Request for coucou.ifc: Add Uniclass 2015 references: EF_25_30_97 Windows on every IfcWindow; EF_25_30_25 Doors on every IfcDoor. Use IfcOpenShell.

First a look at what the model holds.

```python
import ifcopenshell

model = ifcopenshell.open("coucou.ifc")
print(model.schema)
print("classifications:", [c.Name for c in model.by_type("IfcClassification")])
for ifc_class in ("IfcDoor", "IfcRoof", "IfcStair", "IfcWall", "IfcWindow"):
    print(ifc_class, len(model.by_type(ifc_class)))
```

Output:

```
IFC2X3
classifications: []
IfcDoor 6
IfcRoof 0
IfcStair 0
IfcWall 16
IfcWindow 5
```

```python
import ifcopenshell
import ifcopenshell.api.classification

model = ifcopenshell.open("coucou.ifc")

# IFC2X3 requires Source and Edition and has no link from the project to the system.
system = model.create_entity("IfcClassification", Source="NBS", Edition="2015", Name="Uniclass 2015")

codes = {
    "IfcWindow": ("EF_25_30_97", "Windows"),
    "IfcDoor": ("EF_25_30_25", "Doors"),
}
for ifc_class, (code, name) in codes.items():
    products = model.by_type(ifc_class)
    ifcopenshell.api.classification.add_reference(
        model, products=products, classification=system, identification=code, name=name
    )
    print(code, len(products))

model.write("coucou_edited.ifc")
```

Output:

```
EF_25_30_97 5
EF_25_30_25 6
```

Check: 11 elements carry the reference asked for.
